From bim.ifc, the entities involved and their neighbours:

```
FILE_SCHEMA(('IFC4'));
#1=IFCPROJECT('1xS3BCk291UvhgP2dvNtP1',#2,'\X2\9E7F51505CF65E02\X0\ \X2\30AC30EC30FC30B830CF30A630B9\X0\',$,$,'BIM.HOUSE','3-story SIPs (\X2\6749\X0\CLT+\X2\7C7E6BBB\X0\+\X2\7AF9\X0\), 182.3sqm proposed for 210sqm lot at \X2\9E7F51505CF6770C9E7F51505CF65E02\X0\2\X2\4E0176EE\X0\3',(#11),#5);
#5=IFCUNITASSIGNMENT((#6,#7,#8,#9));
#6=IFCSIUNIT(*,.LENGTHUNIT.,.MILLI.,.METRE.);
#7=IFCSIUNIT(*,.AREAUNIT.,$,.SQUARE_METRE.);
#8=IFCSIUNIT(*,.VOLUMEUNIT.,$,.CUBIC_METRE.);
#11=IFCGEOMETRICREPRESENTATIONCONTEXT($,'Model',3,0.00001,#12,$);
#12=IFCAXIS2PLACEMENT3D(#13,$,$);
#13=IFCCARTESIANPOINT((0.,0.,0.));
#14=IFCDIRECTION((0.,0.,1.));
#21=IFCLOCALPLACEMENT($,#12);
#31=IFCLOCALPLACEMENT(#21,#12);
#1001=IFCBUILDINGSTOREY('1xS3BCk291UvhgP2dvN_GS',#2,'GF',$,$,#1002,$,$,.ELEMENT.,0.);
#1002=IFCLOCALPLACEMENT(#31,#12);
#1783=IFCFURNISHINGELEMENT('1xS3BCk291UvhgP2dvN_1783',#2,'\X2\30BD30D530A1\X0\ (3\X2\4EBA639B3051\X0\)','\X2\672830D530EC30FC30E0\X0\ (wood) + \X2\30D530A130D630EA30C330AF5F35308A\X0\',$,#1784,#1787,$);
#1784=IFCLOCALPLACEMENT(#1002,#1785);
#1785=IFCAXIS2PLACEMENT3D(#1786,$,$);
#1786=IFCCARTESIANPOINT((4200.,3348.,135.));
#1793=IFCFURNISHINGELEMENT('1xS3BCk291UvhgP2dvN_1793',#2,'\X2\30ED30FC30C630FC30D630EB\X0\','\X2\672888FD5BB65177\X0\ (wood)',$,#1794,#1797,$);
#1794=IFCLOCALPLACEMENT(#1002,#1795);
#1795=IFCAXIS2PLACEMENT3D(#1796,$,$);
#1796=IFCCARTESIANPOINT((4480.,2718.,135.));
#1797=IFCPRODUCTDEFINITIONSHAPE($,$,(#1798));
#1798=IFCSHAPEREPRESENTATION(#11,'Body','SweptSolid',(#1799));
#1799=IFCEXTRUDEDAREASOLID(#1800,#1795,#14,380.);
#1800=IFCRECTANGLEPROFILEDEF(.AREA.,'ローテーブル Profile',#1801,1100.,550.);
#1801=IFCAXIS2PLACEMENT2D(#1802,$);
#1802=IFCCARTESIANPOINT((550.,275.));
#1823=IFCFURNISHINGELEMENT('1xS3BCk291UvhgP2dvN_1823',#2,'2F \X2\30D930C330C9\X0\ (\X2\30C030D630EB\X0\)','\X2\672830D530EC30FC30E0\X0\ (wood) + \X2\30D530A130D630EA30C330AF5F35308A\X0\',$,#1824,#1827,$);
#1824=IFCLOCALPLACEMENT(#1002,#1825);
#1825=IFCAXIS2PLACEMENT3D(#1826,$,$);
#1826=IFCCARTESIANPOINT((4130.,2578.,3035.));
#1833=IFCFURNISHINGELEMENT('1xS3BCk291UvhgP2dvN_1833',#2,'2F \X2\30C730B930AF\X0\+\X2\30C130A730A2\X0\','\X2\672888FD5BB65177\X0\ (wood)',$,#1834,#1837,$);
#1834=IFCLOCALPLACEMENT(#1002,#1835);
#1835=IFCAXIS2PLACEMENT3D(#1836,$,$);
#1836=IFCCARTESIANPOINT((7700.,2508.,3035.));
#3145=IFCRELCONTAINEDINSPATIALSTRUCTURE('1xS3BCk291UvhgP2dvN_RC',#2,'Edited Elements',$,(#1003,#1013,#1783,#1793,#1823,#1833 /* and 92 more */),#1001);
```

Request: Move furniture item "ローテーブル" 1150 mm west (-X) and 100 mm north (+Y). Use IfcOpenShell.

```python
import ifcopenshell
import ifcopenshell.api.geometry
import ifcopenshell.util.placement

model = ifcopenshell.open("bim.ifc")

item = model.by_id(1793)
matrix = ifcopenshell.util.placement.get_local_placement(item.ObjectPlacement)
matrix[0, 3] -= 1150.0
matrix[1, 3] += 100.0
ifcopenshell.api.geometry.edit_object_placement(model, product=item, matrix=matrix, is_si=False)

print(ifcopenshell.util.placement.get_local_placement(item.ObjectPlacement).round(3) + 0.0)

model.write("bim-out.ifc")
```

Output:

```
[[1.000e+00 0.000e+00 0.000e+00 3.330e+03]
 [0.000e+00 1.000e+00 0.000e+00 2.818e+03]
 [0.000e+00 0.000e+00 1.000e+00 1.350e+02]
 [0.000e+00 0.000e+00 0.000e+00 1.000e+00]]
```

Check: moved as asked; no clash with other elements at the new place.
